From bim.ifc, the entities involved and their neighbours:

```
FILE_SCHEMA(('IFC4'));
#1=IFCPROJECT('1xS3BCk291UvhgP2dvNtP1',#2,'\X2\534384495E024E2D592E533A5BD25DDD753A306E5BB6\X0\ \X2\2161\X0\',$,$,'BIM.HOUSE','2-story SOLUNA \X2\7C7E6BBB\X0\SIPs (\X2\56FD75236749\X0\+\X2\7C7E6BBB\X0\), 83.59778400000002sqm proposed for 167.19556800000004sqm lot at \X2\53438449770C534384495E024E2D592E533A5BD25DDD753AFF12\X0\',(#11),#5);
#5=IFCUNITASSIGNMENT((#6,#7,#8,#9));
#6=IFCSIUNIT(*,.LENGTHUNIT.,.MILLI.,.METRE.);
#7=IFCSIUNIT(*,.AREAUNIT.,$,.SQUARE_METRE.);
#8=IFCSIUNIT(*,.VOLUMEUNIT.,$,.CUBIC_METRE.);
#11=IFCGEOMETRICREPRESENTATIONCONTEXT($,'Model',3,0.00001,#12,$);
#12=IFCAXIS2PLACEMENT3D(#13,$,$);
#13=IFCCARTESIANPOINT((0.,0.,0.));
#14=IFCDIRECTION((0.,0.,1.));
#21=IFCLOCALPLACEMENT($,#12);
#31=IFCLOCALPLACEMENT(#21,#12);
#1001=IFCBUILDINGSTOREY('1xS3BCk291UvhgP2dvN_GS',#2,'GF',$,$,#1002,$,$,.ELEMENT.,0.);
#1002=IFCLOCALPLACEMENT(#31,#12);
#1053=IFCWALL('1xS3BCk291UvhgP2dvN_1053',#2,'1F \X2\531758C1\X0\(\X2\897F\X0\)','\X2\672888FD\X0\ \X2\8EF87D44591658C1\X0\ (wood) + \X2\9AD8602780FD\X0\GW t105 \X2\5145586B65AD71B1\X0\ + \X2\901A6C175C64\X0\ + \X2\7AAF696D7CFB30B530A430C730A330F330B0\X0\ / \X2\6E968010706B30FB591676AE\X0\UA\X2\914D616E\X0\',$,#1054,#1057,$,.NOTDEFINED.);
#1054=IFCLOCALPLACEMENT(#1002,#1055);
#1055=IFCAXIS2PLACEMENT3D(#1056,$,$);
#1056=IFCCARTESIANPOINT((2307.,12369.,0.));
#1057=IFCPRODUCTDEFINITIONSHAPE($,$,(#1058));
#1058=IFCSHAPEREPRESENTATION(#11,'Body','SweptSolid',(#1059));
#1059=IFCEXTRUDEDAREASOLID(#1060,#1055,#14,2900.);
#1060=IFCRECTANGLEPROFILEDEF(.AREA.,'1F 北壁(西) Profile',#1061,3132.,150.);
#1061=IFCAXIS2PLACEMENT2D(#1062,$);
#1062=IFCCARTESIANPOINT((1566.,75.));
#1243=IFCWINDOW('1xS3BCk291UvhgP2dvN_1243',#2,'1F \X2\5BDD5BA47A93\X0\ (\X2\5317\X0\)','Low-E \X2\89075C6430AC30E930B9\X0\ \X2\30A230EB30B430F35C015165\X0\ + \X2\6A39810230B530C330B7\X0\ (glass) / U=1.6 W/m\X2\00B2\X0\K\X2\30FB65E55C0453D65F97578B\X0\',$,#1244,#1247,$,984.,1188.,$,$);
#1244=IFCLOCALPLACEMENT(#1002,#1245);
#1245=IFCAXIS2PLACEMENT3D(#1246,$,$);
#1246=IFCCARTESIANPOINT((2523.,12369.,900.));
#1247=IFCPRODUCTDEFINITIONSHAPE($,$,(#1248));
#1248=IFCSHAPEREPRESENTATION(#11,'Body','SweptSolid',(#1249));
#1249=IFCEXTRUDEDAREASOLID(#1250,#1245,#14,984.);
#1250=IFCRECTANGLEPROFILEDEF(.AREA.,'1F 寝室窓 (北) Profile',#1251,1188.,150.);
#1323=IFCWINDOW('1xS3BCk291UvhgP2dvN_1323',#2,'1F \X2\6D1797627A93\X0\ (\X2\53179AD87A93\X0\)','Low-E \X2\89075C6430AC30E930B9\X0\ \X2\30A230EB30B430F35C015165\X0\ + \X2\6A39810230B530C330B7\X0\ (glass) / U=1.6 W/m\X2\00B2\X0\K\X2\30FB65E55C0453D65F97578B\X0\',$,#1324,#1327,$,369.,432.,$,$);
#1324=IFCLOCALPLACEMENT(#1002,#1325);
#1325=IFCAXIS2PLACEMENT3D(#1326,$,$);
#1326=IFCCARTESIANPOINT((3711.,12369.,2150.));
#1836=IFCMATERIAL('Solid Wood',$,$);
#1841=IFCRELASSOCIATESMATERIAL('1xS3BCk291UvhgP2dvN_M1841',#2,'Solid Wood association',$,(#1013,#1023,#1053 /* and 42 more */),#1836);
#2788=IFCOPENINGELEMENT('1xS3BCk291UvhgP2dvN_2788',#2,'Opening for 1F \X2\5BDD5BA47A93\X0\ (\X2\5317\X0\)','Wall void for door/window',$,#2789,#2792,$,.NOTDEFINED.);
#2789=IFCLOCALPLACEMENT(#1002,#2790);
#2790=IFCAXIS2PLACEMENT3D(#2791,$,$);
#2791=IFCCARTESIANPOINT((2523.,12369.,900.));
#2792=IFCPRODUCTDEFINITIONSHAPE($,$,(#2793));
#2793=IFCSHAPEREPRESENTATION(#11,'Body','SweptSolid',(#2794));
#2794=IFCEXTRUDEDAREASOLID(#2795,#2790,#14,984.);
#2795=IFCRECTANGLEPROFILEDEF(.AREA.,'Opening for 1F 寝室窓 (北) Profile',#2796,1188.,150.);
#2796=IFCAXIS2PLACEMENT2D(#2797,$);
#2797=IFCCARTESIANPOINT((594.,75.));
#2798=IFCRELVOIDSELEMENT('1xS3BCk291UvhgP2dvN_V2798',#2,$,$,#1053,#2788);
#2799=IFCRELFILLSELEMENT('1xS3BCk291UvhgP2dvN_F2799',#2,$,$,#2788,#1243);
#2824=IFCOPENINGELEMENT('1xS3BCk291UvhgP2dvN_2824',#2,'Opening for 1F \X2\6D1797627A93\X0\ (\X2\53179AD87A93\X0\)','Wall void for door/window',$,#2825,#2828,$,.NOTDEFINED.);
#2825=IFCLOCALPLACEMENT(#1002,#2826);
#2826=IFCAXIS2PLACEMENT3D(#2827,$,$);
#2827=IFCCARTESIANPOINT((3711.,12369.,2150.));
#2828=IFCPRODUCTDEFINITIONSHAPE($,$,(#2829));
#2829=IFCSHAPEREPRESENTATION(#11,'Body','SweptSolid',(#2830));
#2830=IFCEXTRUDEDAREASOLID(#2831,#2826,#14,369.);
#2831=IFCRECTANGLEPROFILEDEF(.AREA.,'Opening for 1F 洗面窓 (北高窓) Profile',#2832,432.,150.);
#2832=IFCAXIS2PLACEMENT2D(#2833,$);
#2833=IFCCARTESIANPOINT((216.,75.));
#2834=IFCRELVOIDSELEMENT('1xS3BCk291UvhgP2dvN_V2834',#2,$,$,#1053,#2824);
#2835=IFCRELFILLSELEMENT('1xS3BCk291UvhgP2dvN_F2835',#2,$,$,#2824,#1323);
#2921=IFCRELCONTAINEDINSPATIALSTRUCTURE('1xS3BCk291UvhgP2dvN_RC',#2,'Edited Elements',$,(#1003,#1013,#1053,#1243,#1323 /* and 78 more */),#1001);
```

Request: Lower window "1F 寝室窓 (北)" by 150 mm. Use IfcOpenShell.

```python
import numpy as np
import ifcopenshell
import ifcopenshell.api.geometry
import ifcopenshell.util.placement
import ifcopenshell.util.unit

model = ifcopenshell.open("bim.ifc")
unit_scale = ifcopenshell.util.unit.calculate_unit_scale(model)

window = model.by_guid("1xS3BCk291UvhgP2dvN_1243")
opening = window.FillsVoids[0].RelatingOpeningElement
dz = -0.15 / unit_scale

shift = np.array([0.0, 0.0, dz])
# The window is not placed relative to its opening, so move both.
for product in (opening, window):
    matrix = ifcopenshell.util.placement.get_local_placement(product.ObjectPlacement)
    matrix[:3, 3] += shift
    ifcopenshell.api.geometry.edit_object_placement(model, product=product, matrix=matrix, is_si=False)

print(f"moved by {dz * unit_scale:+.3f} m")

model.write("bim_rev.ifc")
```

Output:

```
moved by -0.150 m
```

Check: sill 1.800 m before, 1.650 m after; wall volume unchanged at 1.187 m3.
